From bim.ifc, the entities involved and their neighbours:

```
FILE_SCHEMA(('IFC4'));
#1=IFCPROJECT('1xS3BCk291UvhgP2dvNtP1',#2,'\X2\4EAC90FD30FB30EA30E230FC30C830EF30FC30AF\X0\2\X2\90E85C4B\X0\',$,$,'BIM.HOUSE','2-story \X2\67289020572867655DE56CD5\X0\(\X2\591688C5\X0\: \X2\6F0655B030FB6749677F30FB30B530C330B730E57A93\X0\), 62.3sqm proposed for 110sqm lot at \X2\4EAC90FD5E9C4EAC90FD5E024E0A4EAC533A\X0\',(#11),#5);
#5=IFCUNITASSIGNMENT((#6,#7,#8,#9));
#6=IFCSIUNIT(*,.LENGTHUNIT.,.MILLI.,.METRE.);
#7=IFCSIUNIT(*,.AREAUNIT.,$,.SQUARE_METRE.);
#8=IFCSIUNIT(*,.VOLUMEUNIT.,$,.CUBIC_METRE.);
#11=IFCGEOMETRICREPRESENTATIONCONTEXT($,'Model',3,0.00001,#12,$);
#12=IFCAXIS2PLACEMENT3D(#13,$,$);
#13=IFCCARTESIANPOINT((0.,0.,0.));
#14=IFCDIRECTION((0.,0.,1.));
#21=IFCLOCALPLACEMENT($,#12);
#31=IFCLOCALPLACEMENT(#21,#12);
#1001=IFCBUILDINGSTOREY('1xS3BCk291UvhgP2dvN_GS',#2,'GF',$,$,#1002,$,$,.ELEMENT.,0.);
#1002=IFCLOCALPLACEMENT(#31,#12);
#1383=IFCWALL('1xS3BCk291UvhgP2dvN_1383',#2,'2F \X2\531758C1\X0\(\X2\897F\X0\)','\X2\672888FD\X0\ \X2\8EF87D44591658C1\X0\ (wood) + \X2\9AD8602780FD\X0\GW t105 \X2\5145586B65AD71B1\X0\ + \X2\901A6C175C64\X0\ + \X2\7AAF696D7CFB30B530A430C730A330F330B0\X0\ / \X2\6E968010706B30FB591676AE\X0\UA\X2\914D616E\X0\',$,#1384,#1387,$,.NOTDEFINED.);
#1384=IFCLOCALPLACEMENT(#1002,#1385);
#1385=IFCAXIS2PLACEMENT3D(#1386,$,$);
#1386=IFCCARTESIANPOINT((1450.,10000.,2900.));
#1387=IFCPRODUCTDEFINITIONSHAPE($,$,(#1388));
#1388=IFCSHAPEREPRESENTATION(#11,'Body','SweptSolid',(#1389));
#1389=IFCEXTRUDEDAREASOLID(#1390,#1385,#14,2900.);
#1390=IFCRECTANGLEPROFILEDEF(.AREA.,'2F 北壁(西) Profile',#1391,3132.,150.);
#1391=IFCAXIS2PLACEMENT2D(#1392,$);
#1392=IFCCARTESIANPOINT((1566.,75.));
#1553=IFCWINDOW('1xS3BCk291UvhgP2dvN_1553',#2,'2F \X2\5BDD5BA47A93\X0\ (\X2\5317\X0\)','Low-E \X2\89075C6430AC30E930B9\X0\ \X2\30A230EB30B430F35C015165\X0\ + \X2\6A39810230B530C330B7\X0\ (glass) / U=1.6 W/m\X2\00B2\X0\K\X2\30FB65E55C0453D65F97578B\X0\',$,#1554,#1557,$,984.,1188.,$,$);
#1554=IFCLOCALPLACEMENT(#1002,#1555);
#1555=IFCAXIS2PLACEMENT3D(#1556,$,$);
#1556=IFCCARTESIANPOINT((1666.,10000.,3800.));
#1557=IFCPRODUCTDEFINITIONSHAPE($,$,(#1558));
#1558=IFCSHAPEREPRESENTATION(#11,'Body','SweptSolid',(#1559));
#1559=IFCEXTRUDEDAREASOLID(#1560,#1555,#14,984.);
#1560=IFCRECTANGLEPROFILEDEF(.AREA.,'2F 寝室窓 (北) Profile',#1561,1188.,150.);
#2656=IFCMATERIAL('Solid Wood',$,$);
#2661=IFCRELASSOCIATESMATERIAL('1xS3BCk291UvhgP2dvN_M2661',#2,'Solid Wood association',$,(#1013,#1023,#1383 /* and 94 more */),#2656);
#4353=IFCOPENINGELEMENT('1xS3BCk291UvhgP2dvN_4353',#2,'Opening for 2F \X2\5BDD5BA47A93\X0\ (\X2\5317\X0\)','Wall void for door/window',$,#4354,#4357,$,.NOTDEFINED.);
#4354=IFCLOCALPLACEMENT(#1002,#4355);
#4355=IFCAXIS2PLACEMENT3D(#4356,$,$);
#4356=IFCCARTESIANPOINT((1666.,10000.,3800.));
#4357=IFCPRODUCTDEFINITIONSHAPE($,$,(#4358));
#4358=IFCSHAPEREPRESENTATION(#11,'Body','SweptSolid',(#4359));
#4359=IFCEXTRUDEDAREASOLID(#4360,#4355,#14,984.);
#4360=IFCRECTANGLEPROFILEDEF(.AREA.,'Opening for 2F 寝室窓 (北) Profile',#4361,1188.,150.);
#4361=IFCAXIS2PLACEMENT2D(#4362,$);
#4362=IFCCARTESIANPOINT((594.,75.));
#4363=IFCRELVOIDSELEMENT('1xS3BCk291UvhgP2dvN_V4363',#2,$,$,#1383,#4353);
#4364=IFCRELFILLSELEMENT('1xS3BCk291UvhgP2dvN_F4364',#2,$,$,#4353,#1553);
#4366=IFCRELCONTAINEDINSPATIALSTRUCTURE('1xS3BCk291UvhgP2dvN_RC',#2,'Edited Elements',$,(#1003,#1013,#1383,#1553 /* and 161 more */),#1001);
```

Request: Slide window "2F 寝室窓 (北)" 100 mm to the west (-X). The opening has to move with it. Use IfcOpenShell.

```python
import ifcopenshell
import ifcopenshell.api.geometry
import ifcopenshell.util.placement

model = ifcopenshell.open("bim.ifc")

window = model.by_id(1553)
opening = window.FillsVoids[0].RelatingOpeningElement
wall = opening.VoidsElements[0].RelatingBuildingElement

wall_matrix = ifcopenshell.util.placement.get_local_placement(wall.ObjectPlacement)
shift = wall_matrix[:3, 0] * -100.0
before = ifcopenshell.util.placement.get_local_placement(window.ObjectPlacement)[:3, 3].copy()

# The window is not placed relative to its opening, so move both.
for product in (opening, window):
    matrix = ifcopenshell.util.placement.get_local_placement(product.ObjectPlacement)
    matrix[:3, 3] += shift
    ifcopenshell.api.geometry.edit_object_placement(model, product=product, matrix=matrix, is_si=False)

after = ifcopenshell.util.placement.get_local_placement(window.ObjectPlacement)[:3, 3]
print("window moved by", (after - before).round(3) + 0.0)

model.write("bim_rev.ifc")
```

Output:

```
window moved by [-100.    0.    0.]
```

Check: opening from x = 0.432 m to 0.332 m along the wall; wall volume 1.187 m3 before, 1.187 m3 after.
